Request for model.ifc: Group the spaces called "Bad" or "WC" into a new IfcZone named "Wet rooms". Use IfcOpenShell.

First a look at what the model holds.

```python
import ifcopenshell

model = ifcopenshell.open("model.ifc")
print(model.schema)
seen = {}
for space in model.by_type("IfcSpace"):
    seen[space.LongName] = seen.get(space.LongName, 0) + 1
for name, count in sorted(seen.items(), key=str):
    print(count, "x", name)
print("zones:", [z.Name for z in model.by_type("IfcZone")][:20])
```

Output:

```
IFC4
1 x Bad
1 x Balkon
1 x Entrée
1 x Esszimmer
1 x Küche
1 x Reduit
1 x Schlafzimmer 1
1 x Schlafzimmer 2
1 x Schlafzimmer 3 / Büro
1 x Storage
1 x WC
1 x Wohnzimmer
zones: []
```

```python
import ifcopenshell
import ifcopenshell.api.group
import ifcopenshell.api.root

model = ifcopenshell.open("model.ifc")

names = {"Bad", "WC"}
spaces = [s for s in model.by_type("IfcSpace") if s.LongName in names]

zone = ifcopenshell.api.root.create_entity(model, ifc_class="IfcZone", name="Wet rooms")
ifcopenshell.api.group.assign_group(model, products=spaces, group=zone)
print(len(spaces), "spaces in", zone.Name)

model.write("model-out.ifc")
```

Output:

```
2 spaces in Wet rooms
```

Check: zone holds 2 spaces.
